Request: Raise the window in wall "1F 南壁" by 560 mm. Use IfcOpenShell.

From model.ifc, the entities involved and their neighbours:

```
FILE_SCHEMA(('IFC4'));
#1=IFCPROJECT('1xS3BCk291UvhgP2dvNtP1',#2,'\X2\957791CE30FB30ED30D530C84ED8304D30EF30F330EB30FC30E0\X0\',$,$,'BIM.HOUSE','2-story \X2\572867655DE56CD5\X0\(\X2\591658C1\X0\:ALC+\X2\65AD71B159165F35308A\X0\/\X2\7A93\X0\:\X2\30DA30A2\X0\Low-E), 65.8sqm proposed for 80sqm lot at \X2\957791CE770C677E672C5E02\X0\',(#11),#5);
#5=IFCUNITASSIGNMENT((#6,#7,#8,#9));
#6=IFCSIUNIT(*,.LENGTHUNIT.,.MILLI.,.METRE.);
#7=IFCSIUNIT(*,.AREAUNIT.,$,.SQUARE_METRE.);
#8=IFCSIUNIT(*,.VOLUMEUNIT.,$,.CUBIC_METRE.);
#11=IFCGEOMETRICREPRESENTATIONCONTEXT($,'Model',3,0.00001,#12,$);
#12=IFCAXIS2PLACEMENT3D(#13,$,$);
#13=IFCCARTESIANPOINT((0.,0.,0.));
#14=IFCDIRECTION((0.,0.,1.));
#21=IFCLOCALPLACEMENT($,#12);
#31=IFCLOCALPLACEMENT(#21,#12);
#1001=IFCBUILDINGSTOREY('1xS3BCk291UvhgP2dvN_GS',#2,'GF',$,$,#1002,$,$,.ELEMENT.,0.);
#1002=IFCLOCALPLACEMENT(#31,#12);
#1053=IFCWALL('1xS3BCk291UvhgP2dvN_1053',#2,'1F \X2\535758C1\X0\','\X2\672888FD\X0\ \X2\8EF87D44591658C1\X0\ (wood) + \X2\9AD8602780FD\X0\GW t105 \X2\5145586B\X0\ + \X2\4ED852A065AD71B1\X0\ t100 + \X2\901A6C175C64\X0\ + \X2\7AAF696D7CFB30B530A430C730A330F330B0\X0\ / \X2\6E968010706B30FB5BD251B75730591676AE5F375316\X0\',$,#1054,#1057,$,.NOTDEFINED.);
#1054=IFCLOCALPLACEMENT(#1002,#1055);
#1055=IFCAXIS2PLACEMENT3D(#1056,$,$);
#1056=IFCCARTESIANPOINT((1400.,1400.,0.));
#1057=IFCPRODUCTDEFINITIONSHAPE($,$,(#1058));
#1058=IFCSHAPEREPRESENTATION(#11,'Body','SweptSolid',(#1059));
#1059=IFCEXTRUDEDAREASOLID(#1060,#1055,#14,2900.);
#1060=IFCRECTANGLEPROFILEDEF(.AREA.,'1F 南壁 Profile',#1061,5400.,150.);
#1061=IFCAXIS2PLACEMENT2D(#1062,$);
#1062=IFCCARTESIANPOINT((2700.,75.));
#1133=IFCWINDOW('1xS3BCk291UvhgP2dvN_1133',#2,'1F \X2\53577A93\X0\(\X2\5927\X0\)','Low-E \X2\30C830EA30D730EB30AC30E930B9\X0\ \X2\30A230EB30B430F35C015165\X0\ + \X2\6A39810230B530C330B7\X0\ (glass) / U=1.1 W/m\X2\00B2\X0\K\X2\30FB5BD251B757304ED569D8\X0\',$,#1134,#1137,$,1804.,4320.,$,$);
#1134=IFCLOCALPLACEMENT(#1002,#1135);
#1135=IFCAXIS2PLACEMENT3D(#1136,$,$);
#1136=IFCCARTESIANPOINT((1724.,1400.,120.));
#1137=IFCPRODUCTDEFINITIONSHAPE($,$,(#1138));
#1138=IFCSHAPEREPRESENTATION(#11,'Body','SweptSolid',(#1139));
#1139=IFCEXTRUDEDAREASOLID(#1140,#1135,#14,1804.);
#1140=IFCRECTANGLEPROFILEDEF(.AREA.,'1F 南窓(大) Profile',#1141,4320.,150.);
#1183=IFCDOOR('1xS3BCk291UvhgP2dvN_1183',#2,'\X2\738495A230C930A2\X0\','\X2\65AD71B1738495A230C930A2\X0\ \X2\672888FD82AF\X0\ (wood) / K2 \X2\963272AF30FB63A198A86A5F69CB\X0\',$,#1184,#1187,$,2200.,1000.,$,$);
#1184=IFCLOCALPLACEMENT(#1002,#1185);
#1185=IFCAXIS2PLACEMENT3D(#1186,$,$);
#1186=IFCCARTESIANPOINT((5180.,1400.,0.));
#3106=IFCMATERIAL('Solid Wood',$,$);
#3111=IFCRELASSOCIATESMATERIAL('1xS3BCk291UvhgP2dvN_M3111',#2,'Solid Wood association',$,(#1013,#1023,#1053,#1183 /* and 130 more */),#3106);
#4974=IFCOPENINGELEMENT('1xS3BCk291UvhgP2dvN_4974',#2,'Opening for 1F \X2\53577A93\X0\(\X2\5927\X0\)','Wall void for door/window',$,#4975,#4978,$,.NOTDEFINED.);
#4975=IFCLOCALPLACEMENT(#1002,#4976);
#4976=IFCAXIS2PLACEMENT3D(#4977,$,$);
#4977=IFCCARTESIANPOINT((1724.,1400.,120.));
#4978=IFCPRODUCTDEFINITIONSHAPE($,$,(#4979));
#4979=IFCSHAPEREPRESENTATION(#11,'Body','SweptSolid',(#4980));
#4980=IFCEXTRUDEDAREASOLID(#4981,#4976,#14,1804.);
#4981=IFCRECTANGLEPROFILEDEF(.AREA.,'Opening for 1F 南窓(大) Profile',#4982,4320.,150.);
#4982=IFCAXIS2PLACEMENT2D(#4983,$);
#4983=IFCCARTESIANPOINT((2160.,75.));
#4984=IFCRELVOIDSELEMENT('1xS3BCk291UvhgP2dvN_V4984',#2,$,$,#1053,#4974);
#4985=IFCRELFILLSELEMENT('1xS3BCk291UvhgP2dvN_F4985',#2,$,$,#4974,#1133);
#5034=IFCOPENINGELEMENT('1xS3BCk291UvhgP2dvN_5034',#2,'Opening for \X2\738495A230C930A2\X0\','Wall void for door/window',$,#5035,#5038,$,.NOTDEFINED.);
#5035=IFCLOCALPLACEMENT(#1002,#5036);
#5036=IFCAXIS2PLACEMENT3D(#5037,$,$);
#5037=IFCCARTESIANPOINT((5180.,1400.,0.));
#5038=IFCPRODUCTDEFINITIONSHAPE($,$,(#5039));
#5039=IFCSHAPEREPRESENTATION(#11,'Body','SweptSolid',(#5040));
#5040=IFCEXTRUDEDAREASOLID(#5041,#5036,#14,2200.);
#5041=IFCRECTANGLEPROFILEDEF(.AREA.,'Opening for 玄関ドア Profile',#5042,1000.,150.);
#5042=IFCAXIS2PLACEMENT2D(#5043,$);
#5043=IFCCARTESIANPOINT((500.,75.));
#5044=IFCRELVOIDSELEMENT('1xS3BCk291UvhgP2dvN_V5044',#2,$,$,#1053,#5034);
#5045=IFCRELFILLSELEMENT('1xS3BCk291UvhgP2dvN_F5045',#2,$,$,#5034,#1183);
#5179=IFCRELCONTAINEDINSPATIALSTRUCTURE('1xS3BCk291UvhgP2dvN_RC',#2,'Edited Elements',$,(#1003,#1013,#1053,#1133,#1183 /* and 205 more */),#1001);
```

```python
import numpy as np
import ifcopenshell
import ifcopenshell.api.geometry
import ifcopenshell.util.placement
import ifcopenshell.util.unit

model = ifcopenshell.open("model.ifc")
unit_scale = ifcopenshell.util.unit.calculate_unit_scale(model)

window = model.by_id(1133)
opening = window.FillsVoids[0].RelatingOpeningElement
dz = 560.0

shift = np.array([0.0, 0.0, dz])
# The window is not placed relative to its opening, so move both.
for product in (opening, window):
    matrix = ifcopenshell.util.placement.get_local_placement(product.ObjectPlacement)
    matrix[:3, 3] += shift
    ifcopenshell.api.geometry.edit_object_placement(model, product=product, matrix=matrix, is_si=False)

print(f"moved by {dz * unit_scale:+.3f} m")

model.write("model-out.ifc")
```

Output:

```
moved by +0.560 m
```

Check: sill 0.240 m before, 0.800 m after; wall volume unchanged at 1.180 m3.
